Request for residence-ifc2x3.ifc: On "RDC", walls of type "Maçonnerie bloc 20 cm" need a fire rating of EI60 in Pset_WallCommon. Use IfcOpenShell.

First a look at what the model holds.

```python
import ifcopenshell
import ifcopenshell.util.element

model = ifcopenshell.open("residence-ifc2x3.ifc")
print(model.schema)
storey = next(s for s in model.by_type("IfcBuildingStorey") if s.Name == "RDC")
walls = [e for e in ifcopenshell.util.element.get_decomposition(storey) if e.is_a("IfcWall")]
seen = {}
for e in walls:
    element_type = ifcopenshell.util.element.get_type(e)
    key = (element_type.Name if element_type != e and element_type else None, ifcopenshell.util.element.get_pset(e, "Pset_WallCommon", "FireRating"))
    seen[key] = seen.get(key, 0) + 1
for (name, value), count in sorted(seen.items(), key=str):
    print(count, "x", name, "|", value)
```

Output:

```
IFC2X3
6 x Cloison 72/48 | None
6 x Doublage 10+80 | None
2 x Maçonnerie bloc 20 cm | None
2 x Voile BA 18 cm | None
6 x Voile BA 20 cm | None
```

```python
import ifcopenshell
import ifcopenshell.api.pset
import ifcopenshell.util.element

model = ifcopenshell.open("residence-ifc2x3.ifc")

storey = next(s for s in model.by_type("IfcBuildingStorey") if s.Name == "RDC")
walls = [e for e in ifcopenshell.util.element.get_decomposition(storey) if e.is_a("IfcWall")]

count = 0
for e in walls:
    element_type = ifcopenshell.util.element.get_type(e)
    if element_type in (None, e) or element_type.Name != "Maçonnerie bloc 20 cm":
        continue
    # add_pset returns the element's existing set when there is one.
    pset = ifcopenshell.api.pset.add_pset(model, product=e, name="Pset_WallCommon")
    ifcopenshell.api.pset.edit_pset(model, pset=pset, properties={"FireRating": "EI60"})
    count += 1

print(count, "walls updated")

model.write("residence-ifc2x3_v2.ifc")
```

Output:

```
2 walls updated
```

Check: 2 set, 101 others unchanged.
